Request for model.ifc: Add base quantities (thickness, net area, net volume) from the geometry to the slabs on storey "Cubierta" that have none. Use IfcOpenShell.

First a look at what the model holds.

```python
import ifcopenshell
import ifcopenshell.util.element
import ifcopenshell.util.unit

model = ifcopenshell.open("model.ifc")
print(model.schema)
for unit_type in ("LENGTHUNIT", "AREAUNIT", "VOLUMEUNIT"):
    print(unit_type, ifcopenshell.util.unit.calculate_unit_scale(model, unit_type))
storey = next(s for s in model.by_type("IfcBuildingStorey") if s.Name == "Cubierta")
slabs = [e for e in ifcopenshell.util.element.get_decomposition(storey) if e.is_a("IfcSlab")]
for e in sorted(slabs, key=lambda e: e.id()):
    print(e.id(), e.is_a(), e.Name, list(ifcopenshell.util.element.get_psets(e, qtos_only=True)), sep=" | ")
```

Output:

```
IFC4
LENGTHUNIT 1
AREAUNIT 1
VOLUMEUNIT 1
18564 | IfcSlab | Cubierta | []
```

```python
import ifcopenshell
import ifcopenshell.api.pset
import ifcopenshell.geom
import ifcopenshell.util.element
import ifcopenshell.util.shape
import ifcopenshell.util.unit

model = ifcopenshell.open("model.ifc")
unit_scale = ifcopenshell.util.unit.calculate_unit_scale(model)
area_scale = ifcopenshell.util.unit.calculate_unit_scale(model, "AREAUNIT")
volume_scale = ifcopenshell.util.unit.calculate_unit_scale(model, "VOLUMEUNIT")
settings = ifcopenshell.geom.settings()

storey = next(s for s in model.by_type("IfcBuildingStorey") if s.Name == "Cubierta")
slabs = [e for e in ifcopenshell.util.element.get_decomposition(storey) if e.is_a("IfcSlab")]

for e in sorted(slabs, key=lambda e: e.id()):
    if ifcopenshell.util.element.get_psets(e, qtos_only=True, should_inherit=False):
        continue
    # Geometry comes back in metres, in the element's own axes.
    shape = ifcopenshell.geom.create_shape(settings, e)
    values = {
        "Width": ifcopenshell.util.shape.get_z(shape.geometry) / unit_scale,
        "NetArea": ifcopenshell.util.shape.get_footprint_area(shape.geometry) / area_scale,
        "NetVolume": ifcopenshell.util.shape.get_volume(shape.geometry) / volume_scale,
    }
    qto = ifcopenshell.api.pset.add_qto(model, product=e, name="Qto_SlabBaseQuantities")
    ifcopenshell.api.pset.edit_qto(model, qto=qto, properties=values)
    print(e.id(), {k: round(v, 3) for k, v in values.items()})

model.write("model_v2.ifc")
```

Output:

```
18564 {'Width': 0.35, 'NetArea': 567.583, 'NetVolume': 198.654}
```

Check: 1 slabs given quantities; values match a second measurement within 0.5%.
